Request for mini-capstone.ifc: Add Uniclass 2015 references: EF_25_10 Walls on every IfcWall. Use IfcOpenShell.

First a look at what the model holds.

```python
import ifcopenshell

model = ifcopenshell.open("mini-capstone.ifc")
print(model.schema)
print("classifications:", [c.Name for c in model.by_type("IfcClassification")])
for ifc_class in ("IfcDoor", "IfcRoof", "IfcStair", "IfcWall", "IfcWindow"):
    print(ifc_class, len(model.by_type(ifc_class)))
```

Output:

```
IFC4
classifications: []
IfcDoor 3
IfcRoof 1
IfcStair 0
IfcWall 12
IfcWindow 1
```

```python
import ifcopenshell
import ifcopenshell.api.classification

model = ifcopenshell.open("mini-capstone.ifc")

system = ifcopenshell.api.classification.add_classification(model, classification="Uniclass 2015")

codes = {
    "IfcWall": ("EF_25_10", "Walls"),
}
for ifc_class, (code, name) in codes.items():
    products = model.by_type(ifc_class)
    ifcopenshell.api.classification.add_reference(
        model, products=products, classification=system, identification=code, name=name
    )
    print(code, len(products))

model.write("mini-capstone_updated.ifc")
```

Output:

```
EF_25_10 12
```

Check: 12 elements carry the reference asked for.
